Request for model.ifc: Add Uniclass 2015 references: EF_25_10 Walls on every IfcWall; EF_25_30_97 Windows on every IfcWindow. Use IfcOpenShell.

First a look at what the model holds.

```python
import ifcopenshell

model = ifcopenshell.open("model.ifc")
print(model.schema)
print("classifications:", [c.Name for c in model.by_type("IfcClassification")])
for ifc_class in ("IfcDoor", "IfcRoof", "IfcStair", "IfcWall", "IfcWindow"):
    print(ifc_class, len(model.by_type(ifc_class)))
```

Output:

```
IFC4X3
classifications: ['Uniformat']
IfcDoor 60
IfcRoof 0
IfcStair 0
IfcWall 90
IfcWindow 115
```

```python
import ifcopenshell
import ifcopenshell.api.classification

model = ifcopenshell.open("model.ifc")

system = ifcopenshell.api.classification.add_classification(model, classification="Uniclass 2015")

codes = {
    "IfcWall": ("EF_25_10", "Walls"),
    "IfcWindow": ("EF_25_30_97", "Windows"),
}
for ifc_class, (code, name) in codes.items():
    products = model.by_type(ifc_class)
    ifcopenshell.api.classification.add_reference(
        model, products=products, classification=system, identification=code, name=name
    )
    print(code, len(products))

model.write("model_rev.ifc")
```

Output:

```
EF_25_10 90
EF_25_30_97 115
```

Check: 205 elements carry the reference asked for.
